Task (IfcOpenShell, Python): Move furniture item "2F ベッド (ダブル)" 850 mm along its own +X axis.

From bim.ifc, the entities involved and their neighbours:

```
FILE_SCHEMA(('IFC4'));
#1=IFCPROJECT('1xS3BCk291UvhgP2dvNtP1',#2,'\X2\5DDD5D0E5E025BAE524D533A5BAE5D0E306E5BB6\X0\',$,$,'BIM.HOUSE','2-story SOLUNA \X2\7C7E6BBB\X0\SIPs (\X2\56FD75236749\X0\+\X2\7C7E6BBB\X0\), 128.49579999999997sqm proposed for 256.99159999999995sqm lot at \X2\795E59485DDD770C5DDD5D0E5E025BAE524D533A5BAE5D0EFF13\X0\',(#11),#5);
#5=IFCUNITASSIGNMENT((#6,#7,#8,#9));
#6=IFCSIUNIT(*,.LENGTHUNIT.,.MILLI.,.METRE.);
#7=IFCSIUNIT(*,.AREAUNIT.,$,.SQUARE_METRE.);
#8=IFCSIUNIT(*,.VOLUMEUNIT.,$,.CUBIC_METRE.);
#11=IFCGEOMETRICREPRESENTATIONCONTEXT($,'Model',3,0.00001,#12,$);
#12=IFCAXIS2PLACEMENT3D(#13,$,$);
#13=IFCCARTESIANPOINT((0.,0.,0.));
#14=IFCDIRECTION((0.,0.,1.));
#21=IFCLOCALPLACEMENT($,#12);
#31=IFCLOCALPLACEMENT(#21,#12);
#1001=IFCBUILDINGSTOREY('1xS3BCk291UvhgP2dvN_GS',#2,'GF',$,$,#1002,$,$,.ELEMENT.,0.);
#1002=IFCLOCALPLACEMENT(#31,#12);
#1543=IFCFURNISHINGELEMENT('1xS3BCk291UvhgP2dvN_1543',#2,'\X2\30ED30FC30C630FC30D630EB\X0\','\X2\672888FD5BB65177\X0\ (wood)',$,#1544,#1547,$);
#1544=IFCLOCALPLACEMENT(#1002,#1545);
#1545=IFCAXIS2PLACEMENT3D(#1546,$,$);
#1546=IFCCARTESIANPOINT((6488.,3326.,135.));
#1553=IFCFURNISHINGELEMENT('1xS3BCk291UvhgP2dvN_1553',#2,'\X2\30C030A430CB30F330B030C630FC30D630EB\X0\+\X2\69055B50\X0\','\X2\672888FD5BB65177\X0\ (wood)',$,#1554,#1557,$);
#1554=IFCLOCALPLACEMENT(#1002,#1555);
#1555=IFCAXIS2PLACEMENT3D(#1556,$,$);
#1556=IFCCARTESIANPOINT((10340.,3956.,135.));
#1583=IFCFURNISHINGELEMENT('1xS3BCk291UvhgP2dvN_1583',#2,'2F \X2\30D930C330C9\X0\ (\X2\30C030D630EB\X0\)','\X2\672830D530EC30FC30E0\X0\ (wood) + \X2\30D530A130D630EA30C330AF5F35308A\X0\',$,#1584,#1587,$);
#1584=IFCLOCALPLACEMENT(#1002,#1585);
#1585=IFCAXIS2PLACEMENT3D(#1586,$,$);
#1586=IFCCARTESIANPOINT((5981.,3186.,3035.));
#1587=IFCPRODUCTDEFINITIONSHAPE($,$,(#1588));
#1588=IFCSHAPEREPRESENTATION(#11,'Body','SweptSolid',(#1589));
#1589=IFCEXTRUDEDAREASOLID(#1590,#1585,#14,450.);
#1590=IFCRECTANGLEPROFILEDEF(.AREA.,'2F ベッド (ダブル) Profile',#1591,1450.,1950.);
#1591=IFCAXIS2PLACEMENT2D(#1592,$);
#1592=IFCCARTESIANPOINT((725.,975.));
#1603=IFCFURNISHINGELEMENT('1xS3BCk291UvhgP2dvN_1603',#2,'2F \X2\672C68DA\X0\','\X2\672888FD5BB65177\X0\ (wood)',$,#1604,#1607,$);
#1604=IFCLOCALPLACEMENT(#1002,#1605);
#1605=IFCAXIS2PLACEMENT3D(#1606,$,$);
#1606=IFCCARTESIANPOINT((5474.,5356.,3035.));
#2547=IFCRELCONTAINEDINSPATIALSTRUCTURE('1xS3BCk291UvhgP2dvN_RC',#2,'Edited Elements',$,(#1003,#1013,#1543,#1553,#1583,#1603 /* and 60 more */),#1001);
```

```python
import ifcopenshell
import ifcopenshell.api.geometry
import ifcopenshell.util.placement
import ifcopenshell.util.unit

model = ifcopenshell.open("bim.ifc")
unit_scale = ifcopenshell.util.unit.calculate_unit_scale(model)

item = model.by_id(1583)
matrix = ifcopenshell.util.placement.get_local_placement(item.ObjectPlacement)
matrix[:3, 3] += matrix[:3, 0] * 0.85 / unit_scale
ifcopenshell.api.geometry.edit_object_placement(model, product=item, matrix=matrix, is_si=False)

print(ifcopenshell.util.placement.get_local_placement(item.ObjectPlacement).round(3) + 0.0)

model.write("bim_v2.ifc")
```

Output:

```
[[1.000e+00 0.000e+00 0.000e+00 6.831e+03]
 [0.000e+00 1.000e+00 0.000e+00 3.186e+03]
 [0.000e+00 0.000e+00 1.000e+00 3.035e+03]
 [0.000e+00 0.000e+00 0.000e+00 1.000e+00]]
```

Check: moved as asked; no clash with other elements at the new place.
